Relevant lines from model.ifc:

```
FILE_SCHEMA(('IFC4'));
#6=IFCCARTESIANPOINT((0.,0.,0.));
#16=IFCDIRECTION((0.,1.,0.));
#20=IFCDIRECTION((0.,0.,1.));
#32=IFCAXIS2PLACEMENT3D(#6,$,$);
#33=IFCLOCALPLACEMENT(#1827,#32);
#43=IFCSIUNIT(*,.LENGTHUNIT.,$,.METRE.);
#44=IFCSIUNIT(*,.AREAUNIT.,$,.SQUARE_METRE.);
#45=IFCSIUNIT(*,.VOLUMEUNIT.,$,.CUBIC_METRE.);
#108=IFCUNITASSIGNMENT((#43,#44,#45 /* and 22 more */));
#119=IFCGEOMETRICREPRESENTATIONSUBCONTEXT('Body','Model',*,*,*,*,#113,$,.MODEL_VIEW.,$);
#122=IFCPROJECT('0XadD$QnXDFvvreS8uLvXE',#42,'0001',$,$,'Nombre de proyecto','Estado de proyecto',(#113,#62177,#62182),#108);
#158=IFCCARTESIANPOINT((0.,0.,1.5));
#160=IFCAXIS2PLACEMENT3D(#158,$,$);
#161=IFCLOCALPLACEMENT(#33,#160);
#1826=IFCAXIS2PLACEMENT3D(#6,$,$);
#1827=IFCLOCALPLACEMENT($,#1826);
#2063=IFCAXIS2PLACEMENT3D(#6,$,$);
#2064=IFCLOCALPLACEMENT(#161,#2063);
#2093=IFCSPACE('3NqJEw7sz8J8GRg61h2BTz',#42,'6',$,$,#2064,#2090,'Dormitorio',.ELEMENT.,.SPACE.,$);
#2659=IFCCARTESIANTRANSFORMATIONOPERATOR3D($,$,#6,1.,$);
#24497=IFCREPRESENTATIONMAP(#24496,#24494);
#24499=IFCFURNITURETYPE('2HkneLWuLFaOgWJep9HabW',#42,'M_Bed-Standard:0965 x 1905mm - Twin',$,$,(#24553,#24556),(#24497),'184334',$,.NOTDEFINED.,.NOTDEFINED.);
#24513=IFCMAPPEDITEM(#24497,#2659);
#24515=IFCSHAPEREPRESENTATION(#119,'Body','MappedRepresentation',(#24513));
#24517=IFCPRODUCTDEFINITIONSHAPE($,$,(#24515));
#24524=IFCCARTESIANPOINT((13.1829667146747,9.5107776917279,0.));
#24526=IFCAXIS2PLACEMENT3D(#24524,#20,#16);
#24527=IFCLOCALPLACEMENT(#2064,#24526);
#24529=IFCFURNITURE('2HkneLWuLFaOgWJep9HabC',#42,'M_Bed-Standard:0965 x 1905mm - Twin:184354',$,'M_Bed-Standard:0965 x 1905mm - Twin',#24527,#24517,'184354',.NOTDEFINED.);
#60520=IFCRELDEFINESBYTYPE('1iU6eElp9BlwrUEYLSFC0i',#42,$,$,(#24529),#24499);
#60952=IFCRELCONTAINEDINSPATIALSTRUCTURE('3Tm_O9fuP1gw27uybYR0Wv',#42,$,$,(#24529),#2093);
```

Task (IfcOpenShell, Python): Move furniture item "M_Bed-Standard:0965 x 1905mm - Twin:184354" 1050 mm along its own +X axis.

```python
import ifcopenshell
import ifcopenshell.api.geometry
import ifcopenshell.util.placement
import ifcopenshell.util.unit

model = ifcopenshell.open("model.ifc")
unit_scale = ifcopenshell.util.unit.calculate_unit_scale(model)

item = model.by_id(24529)
matrix = ifcopenshell.util.placement.get_local_placement(item.ObjectPlacement)
matrix[:3, 3] += matrix[:3, 0] * 1.05 / unit_scale
ifcopenshell.api.geometry.edit_object_placement(model, product=item, matrix=matrix, is_si=False)

print(ifcopenshell.util.placement.get_local_placement(item.ObjectPlacement).round(3) + 0.0)

model.write("model_rev.ifc")
```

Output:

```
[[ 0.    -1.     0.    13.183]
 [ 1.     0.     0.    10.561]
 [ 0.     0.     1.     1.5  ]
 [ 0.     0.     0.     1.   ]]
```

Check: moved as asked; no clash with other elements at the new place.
